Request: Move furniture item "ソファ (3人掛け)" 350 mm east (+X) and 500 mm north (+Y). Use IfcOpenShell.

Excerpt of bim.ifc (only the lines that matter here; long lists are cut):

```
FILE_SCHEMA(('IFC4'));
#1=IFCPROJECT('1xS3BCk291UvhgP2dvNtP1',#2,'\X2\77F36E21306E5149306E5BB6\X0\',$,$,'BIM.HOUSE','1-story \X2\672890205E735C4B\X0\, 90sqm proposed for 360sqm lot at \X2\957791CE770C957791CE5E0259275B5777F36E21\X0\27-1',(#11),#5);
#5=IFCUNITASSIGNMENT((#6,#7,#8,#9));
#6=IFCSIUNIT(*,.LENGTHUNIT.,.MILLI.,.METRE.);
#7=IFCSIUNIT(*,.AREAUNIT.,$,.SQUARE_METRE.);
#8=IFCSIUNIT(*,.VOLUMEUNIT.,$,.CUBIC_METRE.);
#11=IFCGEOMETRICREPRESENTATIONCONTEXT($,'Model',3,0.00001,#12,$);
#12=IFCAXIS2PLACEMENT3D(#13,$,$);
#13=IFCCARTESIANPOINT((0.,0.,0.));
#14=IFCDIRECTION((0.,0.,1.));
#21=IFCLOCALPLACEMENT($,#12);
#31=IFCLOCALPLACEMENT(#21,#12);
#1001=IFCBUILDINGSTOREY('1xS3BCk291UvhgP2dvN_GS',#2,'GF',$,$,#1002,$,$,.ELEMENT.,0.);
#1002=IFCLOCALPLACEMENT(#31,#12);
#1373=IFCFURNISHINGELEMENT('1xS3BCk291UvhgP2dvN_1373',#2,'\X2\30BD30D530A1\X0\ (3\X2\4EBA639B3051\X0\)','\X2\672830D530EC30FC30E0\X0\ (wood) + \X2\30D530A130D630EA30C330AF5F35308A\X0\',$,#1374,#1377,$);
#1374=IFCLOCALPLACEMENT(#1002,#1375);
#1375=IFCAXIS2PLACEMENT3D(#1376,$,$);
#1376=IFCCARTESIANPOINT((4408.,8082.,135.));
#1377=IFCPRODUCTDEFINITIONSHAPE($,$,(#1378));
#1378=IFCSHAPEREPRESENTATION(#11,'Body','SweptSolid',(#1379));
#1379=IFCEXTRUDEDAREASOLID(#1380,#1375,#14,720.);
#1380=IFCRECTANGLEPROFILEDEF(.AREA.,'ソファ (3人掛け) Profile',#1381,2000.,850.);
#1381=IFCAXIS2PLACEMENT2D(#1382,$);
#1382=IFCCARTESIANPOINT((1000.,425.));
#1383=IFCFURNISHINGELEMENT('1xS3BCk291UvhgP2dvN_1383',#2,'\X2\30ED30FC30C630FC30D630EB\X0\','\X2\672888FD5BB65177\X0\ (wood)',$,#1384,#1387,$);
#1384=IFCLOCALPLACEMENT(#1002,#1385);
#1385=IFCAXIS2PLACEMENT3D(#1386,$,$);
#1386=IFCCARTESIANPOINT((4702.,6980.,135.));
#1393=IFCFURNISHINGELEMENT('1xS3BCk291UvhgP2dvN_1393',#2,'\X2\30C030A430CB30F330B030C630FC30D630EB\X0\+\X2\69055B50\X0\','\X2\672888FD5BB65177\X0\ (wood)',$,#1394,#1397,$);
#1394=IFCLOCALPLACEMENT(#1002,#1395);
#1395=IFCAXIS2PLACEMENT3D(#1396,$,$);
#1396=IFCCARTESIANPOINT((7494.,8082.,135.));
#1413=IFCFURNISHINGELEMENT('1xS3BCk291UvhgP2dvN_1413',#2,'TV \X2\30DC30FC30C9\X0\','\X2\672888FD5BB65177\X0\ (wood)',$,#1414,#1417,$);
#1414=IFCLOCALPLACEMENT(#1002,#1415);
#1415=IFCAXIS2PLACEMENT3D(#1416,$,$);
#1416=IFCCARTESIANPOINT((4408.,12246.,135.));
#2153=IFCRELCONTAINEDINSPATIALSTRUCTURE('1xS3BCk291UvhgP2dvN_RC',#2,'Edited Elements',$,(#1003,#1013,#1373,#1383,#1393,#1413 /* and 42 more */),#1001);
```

```python
import ifcopenshell
import ifcopenshell.api.geometry
import ifcopenshell.util.placement
import ifcopenshell.util.unit

model = ifcopenshell.open("bim.ifc")
unit_scale = ifcopenshell.util.unit.calculate_unit_scale(model)

item = model.by_guid("1xS3BCk291UvhgP2dvN_1373")
matrix = ifcopenshell.util.placement.get_local_placement(item.ObjectPlacement)
matrix[0, 3] += 0.35 / unit_scale
matrix[1, 3] += 0.5 / unit_scale
ifcopenshell.api.geometry.edit_object_placement(model, product=item, matrix=matrix, is_si=False)

print(ifcopenshell.util.placement.get_local_placement(item.ObjectPlacement).round(3) + 0.0)

model.write("bim_edited.ifc")
```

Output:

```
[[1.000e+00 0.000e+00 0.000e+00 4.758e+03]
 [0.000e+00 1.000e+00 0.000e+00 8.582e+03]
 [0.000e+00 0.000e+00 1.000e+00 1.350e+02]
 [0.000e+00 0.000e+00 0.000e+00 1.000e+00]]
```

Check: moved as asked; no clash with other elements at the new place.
